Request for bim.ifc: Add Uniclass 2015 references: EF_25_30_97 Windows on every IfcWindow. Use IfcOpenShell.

First a look at what the model holds.

```python
import ifcopenshell

model = ifcopenshell.open("bim.ifc")
print(model.schema)
print("classifications:", [c.Name for c in model.by_type("IfcClassification")])
for ifc_class in ("IfcDoor", "IfcRoof", "IfcStair", "IfcWall", "IfcWindow"):
    print(ifc_class, len(model.by_type(ifc_class)))
```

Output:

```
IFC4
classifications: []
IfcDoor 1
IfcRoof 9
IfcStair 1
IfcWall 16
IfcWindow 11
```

```python
import ifcopenshell
import ifcopenshell.api.classification

model = ifcopenshell.open("bim.ifc")

system = ifcopenshell.api.classification.add_classification(model, classification="Uniclass 2015")

codes = {
    "IfcWindow": ("EF_25_30_97", "Windows"),
}
for ifc_class, (code, name) in codes.items():
    products = model.by_type(ifc_class)
    ifcopenshell.api.classification.add_reference(
        model, products=products, classification=system, identification=code, name=name
    )
    print(code, len(products))

model.write("bim_rev.ifc")
```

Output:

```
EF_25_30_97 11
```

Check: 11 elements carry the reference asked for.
